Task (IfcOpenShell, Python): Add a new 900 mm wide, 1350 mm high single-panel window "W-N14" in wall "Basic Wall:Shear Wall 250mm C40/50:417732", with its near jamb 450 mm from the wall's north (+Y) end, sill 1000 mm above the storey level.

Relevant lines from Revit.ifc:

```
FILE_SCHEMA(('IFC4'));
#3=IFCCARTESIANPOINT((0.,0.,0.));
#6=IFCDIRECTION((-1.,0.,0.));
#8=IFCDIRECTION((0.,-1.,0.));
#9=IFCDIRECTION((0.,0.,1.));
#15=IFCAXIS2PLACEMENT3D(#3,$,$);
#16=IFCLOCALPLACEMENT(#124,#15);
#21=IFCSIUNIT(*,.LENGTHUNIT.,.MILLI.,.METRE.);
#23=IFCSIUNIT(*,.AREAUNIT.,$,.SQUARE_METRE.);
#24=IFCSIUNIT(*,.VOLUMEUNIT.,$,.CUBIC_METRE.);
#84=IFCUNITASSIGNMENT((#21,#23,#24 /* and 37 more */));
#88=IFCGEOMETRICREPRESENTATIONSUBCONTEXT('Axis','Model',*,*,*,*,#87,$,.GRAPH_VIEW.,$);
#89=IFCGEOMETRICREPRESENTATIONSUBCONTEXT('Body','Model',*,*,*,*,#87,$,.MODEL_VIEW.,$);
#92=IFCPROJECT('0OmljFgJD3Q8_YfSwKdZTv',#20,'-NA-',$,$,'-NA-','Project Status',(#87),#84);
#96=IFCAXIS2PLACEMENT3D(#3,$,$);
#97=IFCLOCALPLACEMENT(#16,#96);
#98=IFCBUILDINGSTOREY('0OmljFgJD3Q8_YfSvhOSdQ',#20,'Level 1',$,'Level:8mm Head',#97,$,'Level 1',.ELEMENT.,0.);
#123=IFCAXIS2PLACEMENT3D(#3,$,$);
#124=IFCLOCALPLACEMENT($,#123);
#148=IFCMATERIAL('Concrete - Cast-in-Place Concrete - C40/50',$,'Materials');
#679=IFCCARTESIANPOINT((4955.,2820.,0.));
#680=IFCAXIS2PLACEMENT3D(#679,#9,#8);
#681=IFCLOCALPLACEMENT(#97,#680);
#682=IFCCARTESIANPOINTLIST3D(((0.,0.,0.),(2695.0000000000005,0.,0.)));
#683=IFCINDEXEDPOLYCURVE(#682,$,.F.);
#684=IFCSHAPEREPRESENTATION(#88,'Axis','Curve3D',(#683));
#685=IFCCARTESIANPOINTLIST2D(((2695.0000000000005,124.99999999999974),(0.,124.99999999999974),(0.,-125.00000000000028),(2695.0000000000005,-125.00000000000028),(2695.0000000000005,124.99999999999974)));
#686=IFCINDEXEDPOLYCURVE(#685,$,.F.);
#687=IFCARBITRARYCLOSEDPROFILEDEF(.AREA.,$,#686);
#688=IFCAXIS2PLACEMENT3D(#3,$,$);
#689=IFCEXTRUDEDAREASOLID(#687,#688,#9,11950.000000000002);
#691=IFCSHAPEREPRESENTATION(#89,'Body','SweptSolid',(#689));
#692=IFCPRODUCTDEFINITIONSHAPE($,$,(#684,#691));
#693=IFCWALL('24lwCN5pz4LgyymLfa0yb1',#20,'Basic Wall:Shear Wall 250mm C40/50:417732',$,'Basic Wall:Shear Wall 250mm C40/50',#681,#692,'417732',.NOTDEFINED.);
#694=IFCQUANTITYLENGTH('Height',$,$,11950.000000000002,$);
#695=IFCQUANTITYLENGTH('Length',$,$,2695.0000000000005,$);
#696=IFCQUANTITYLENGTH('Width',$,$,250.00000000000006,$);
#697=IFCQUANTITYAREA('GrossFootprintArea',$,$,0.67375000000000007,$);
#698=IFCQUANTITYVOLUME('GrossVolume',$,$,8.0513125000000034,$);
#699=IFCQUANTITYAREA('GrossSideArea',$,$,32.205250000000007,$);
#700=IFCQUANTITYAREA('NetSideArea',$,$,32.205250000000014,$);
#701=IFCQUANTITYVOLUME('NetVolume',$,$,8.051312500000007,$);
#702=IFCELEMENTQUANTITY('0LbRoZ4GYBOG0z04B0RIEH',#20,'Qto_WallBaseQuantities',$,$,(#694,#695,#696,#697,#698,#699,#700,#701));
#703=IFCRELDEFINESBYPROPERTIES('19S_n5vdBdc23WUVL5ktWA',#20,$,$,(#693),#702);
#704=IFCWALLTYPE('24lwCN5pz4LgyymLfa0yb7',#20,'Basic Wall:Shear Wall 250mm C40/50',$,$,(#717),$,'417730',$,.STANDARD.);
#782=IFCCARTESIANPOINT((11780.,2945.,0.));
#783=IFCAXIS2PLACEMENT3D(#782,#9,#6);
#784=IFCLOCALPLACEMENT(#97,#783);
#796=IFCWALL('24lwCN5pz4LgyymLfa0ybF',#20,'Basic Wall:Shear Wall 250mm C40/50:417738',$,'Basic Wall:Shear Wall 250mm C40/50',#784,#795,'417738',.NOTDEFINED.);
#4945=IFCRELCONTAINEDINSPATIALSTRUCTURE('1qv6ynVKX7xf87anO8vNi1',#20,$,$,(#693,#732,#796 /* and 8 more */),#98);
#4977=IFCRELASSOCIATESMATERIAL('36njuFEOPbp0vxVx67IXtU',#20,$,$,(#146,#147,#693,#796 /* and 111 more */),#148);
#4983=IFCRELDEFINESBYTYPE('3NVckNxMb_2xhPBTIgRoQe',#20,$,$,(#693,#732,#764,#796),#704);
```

```python
import numpy as np
import ifcopenshell
import ifcopenshell.api.feature
import ifcopenshell.api.geometry
import ifcopenshell.api.pset
import ifcopenshell.api.root
import ifcopenshell.api.spatial
import ifcopenshell.geom
import ifcopenshell.util.element
import ifcopenshell.util.placement
import ifcopenshell.util.representation
import ifcopenshell.util.shape
import ifcopenshell.util.unit

model = ifcopenshell.open("Revit.ifc")
unit_scale = ifcopenshell.util.unit.calculate_unit_scale(model)
area_scale = ifcopenshell.util.unit.calculate_unit_scale(model, "AREAUNIT")
volume_scale = ifcopenshell.util.unit.calculate_unit_scale(model, "VOLUMEUNIT")
settings = ifcopenshell.geom.settings()


def volume(element):
    """Net volume in cubic metres, openings subtracted."""
    shape = ifcopenshell.geom.create_shape(settings, element)
    return ifcopenshell.util.shape.get_volume(shape.geometry)


wall = model.by_id(693)
storey = ifcopenshell.util.element.get_container(wall, ifc_class="IfcBuildingStorey")
context = ifcopenshell.util.representation.get_context(model, "Model", "Body", "MODEL_VIEW")
before = volume(wall)

width, height, from_end, sill = 0.9, 1.35, 0.45, 1  # metres

# The wall runs along its own X axis, and the end named is its -X end.
wall_shape = ifcopenshell.geom.create_shape(settings, wall)
x, y, z = ifcopenshell.util.shape.get_vertices(wall_shape.geometry).T
start = x.min() + from_end
face, thickness = float(y.min()), float(y.max() - y.min())
wall_matrix = ifcopenshell.util.placement.get_local_placement(wall.ObjectPlacement)
level = ifcopenshell.util.placement.get_local_placement(storey.ObjectPlacement)[2, 3]


def in_wall(x, y):
    """Placement at x, y metres in the wall's axes, at sill height."""
    matrix = wall_matrix.copy()
    matrix[:, 3] = wall_matrix @ np.array([x / unit_scale, y / unit_scale, 0.0, 1.0])
    matrix[2, 3] = level + sill / unit_scale
    return matrix


# Opening: a box that overshoots both wall faces by 50 mm.
opening = ifcopenshell.api.root.create_entity(model, ifc_class="IfcOpeningElement", predefined_type="OPENING")
box = ifcopenshell.api.geometry.add_wall_representation(
    model, context=context, length=width, height=height, thickness=thickness + 0.1
)
ifcopenshell.api.geometry.assign_representation(model, product=opening, representation=box)
ifcopenshell.api.geometry.edit_object_placement(model, product=opening, matrix=in_wall(start, face - 0.05), is_si=False)
ifcopenshell.api.feature.add_feature(model, feature=opening, element=wall)

window = ifcopenshell.api.root.create_entity(model, ifc_class="IfcWindow", name="W-N14", predefined_type="WINDOW")
window.OverallWidth, window.OverallHeight = width / unit_scale, height / unit_scale
window.PartitioningType = "SINGLE_PANEL"
body = ifcopenshell.api.geometry.add_window_representation(
    model,
    context=context,
    overall_width=window.OverallWidth,
    overall_height=window.OverallHeight,
    partition_type="SINGLE_PANEL",
)
ifcopenshell.api.geometry.assign_representation(model, product=window, representation=body)
ifcopenshell.api.spatial.assign_container(model, products=[window], relating_structure=storey)
ifcopenshell.api.feature.add_filling(model, opening=opening, element=window)

# Centre the window in the wall's thickness.
ifcopenshell.api.geometry.edit_object_placement(model, product=window, matrix=in_wall(start, face), is_si=False)
window_shape = ifcopenshell.geom.create_shape(settings, window)
depth = ifcopenshell.util.shape.get_vertices(window_shape.geometry)[:, 1]
offset = face + thickness / 2 - (depth.min() + depth.max()) / 2
ifcopenshell.api.geometry.edit_object_placement(model, product=window, matrix=in_wall(start, offset), is_si=False)

after = volume(wall)

# Update the wall's stored quantities.
qto = model.by_id(ifcopenshell.util.element.get_pset(wall, "Qto_WallBaseQuantities", should_inherit=False)["id"])
ifcopenshell.api.pset.edit_qto(model, qto=qto, properties={
    "NetSideArea": after / thickness / area_scale,
    "NetVolume": after / volume_scale,
})

print(f"wall volume {before:.3f} -> {after:.3f} m3")

model.write("Revit-out.ifc")
```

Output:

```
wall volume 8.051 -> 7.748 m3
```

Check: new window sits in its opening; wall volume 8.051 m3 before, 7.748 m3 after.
